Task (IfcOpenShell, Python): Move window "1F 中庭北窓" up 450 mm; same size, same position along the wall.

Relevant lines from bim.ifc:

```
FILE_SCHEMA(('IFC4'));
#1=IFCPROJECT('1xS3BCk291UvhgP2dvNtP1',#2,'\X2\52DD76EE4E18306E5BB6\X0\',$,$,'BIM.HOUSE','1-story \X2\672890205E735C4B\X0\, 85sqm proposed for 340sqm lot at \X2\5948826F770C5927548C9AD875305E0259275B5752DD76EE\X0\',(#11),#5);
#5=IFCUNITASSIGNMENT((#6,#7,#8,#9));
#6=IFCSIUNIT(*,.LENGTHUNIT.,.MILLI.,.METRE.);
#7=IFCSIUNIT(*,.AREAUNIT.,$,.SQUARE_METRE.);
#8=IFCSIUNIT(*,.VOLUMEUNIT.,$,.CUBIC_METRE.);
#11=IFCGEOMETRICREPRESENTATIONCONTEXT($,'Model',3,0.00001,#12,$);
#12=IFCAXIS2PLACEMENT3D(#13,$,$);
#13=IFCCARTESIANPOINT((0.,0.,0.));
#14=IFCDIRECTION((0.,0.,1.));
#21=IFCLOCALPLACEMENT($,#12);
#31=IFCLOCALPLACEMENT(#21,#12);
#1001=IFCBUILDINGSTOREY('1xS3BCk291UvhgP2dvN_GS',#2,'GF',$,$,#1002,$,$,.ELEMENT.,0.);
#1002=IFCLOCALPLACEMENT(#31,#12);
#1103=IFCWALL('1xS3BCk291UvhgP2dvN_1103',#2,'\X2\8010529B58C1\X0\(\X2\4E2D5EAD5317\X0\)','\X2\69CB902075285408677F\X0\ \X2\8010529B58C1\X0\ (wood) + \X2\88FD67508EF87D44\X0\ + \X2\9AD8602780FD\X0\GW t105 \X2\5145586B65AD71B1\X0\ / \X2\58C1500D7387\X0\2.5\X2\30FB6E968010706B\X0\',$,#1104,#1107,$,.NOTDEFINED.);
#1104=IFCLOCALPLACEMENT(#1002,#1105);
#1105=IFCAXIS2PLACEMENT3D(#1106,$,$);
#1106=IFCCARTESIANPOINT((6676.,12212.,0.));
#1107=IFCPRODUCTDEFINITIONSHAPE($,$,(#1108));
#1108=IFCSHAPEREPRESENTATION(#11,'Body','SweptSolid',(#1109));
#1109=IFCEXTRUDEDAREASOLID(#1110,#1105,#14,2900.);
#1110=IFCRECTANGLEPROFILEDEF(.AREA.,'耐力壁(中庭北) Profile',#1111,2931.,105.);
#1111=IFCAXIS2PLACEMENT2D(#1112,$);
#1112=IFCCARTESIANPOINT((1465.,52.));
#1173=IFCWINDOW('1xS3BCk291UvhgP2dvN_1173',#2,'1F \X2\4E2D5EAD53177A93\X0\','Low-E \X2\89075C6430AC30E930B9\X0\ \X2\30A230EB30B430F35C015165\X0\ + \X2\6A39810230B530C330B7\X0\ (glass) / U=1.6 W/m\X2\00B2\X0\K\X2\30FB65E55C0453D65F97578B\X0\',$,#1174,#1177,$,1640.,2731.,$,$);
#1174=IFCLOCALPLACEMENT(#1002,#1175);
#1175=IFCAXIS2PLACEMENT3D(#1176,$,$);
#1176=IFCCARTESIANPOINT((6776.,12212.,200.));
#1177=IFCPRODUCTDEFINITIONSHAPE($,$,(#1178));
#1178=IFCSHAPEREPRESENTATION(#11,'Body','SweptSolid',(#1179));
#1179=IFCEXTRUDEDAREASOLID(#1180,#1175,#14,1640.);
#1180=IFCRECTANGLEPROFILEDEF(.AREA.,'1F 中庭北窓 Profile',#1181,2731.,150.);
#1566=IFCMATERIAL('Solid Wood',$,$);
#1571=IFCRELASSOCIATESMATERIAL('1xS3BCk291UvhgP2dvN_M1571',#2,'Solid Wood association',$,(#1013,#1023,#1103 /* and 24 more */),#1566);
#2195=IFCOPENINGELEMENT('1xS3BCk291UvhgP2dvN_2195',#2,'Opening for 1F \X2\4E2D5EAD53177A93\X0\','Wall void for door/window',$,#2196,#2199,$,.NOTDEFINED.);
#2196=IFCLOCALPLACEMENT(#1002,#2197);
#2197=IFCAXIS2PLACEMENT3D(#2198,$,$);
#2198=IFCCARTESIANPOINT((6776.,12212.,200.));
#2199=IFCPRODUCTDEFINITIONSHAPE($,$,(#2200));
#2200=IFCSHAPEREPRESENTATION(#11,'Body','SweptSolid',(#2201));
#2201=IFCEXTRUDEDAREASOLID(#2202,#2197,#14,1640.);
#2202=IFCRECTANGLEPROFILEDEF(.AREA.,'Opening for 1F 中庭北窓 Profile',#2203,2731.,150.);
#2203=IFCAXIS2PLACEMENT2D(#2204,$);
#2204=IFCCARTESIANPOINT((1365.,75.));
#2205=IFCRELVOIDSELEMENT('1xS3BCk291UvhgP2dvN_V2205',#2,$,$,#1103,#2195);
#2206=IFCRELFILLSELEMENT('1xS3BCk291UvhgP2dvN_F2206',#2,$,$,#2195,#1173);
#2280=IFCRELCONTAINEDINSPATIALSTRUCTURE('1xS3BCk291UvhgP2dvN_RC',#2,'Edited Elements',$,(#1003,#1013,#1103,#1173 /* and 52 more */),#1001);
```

```python
import numpy as np
import ifcopenshell
import ifcopenshell.api.geometry
import ifcopenshell.util.placement
import ifcopenshell.util.unit

model = ifcopenshell.open("bim.ifc")
unit_scale = ifcopenshell.util.unit.calculate_unit_scale(model)

window = model.by_id(1173)
opening = window.FillsVoids[0].RelatingOpeningElement
dz = 0.45 / unit_scale

shift = np.array([0.0, 0.0, dz])
# The window is not placed relative to its opening, so move both.
for product in (opening, window):
    matrix = ifcopenshell.util.placement.get_local_placement(product.ObjectPlacement)
    matrix[:3, 3] += shift
    ifcopenshell.api.geometry.edit_object_placement(model, product=product, matrix=matrix, is_si=False)

print(f"moved by {dz * unit_scale:+.3f} m")

model.write("bim_rev.ifc")
```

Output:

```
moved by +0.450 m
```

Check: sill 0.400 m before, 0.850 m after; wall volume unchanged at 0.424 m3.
